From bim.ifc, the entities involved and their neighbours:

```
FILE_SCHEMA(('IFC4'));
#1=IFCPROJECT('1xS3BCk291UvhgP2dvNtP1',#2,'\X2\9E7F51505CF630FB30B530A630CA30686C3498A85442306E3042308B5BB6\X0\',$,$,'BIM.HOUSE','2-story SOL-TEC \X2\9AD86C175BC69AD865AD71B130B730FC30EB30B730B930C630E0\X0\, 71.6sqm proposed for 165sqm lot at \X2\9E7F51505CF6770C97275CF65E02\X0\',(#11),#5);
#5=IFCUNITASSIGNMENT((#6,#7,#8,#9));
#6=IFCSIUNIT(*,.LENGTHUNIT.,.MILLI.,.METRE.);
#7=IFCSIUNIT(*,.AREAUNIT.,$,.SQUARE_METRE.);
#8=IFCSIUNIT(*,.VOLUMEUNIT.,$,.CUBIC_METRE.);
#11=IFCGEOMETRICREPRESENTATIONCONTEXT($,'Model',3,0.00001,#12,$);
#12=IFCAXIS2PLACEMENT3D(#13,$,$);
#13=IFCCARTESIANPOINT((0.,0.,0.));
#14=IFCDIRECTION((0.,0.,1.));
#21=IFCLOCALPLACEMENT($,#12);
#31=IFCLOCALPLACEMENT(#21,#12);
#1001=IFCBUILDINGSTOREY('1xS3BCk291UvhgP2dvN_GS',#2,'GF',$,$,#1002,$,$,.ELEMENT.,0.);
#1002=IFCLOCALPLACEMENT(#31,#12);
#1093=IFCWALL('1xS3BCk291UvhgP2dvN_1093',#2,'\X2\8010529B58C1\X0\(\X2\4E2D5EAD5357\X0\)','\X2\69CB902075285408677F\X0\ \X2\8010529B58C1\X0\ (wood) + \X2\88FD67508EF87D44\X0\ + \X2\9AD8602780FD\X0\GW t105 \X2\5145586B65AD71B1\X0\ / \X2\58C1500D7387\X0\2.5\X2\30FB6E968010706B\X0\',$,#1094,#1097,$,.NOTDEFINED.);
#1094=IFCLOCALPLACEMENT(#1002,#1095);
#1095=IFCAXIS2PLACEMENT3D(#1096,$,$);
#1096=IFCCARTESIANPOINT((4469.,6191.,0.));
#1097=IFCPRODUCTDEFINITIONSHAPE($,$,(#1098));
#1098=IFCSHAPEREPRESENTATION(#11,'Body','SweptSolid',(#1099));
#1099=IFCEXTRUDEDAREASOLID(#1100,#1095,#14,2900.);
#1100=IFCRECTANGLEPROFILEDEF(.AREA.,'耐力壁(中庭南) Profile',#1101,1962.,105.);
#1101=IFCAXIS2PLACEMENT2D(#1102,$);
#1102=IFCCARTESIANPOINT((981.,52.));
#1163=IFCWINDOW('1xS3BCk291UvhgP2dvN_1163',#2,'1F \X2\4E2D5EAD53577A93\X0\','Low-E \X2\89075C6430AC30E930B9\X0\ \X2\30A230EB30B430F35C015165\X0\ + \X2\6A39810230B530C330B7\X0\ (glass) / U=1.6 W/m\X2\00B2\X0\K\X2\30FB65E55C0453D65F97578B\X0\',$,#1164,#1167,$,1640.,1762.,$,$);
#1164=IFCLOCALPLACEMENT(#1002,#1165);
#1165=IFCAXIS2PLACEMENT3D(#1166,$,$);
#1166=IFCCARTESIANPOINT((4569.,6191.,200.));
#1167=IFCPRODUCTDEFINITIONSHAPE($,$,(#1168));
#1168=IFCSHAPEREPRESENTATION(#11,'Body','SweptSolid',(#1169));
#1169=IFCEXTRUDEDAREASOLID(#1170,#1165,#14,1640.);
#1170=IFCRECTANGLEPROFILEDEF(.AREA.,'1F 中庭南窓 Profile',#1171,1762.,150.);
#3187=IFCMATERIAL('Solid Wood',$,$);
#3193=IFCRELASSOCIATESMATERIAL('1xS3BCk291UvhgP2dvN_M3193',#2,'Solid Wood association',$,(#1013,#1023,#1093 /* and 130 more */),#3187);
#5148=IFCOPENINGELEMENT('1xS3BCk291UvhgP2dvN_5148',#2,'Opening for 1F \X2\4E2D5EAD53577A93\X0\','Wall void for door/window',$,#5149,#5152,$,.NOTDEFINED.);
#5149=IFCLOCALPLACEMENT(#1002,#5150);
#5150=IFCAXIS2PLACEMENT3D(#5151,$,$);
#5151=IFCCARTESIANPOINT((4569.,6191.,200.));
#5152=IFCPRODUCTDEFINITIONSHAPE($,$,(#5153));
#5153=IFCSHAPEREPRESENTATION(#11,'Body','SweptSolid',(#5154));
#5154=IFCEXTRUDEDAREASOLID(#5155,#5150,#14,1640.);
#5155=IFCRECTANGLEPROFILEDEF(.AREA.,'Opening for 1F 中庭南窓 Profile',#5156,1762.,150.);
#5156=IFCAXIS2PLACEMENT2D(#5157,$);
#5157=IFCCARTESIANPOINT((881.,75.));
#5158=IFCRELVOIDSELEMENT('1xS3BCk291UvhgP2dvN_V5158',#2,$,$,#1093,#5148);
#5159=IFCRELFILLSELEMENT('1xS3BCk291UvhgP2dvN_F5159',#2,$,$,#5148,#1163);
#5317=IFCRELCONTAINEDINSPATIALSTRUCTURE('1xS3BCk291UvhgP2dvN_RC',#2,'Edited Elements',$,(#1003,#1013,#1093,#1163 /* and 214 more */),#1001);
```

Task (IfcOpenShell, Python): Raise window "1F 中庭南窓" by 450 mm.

```python
import numpy as np
import ifcopenshell
import ifcopenshell.api.geometry
import ifcopenshell.util.placement
import ifcopenshell.util.unit

model = ifcopenshell.open("bim.ifc")
unit_scale = ifcopenshell.util.unit.calculate_unit_scale(model)

window = model.by_id(1163)
opening = window.FillsVoids[0].RelatingOpeningElement
dz = 0.45 / unit_scale

shift = np.array([0.0, 0.0, dz])
# The window is not placed relative to its opening, so move both.
for product in (opening, window):
    matrix = ifcopenshell.util.placement.get_local_placement(product.ObjectPlacement)
    matrix[:3, 3] += shift
    ifcopenshell.api.geometry.edit_object_placement(model, product=product, matrix=matrix, is_si=False)

print(f"moved by {dz * unit_scale:+.3f} m")

model.write("bim-out.ifc")
```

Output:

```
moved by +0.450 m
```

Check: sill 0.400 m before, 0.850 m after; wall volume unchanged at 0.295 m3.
